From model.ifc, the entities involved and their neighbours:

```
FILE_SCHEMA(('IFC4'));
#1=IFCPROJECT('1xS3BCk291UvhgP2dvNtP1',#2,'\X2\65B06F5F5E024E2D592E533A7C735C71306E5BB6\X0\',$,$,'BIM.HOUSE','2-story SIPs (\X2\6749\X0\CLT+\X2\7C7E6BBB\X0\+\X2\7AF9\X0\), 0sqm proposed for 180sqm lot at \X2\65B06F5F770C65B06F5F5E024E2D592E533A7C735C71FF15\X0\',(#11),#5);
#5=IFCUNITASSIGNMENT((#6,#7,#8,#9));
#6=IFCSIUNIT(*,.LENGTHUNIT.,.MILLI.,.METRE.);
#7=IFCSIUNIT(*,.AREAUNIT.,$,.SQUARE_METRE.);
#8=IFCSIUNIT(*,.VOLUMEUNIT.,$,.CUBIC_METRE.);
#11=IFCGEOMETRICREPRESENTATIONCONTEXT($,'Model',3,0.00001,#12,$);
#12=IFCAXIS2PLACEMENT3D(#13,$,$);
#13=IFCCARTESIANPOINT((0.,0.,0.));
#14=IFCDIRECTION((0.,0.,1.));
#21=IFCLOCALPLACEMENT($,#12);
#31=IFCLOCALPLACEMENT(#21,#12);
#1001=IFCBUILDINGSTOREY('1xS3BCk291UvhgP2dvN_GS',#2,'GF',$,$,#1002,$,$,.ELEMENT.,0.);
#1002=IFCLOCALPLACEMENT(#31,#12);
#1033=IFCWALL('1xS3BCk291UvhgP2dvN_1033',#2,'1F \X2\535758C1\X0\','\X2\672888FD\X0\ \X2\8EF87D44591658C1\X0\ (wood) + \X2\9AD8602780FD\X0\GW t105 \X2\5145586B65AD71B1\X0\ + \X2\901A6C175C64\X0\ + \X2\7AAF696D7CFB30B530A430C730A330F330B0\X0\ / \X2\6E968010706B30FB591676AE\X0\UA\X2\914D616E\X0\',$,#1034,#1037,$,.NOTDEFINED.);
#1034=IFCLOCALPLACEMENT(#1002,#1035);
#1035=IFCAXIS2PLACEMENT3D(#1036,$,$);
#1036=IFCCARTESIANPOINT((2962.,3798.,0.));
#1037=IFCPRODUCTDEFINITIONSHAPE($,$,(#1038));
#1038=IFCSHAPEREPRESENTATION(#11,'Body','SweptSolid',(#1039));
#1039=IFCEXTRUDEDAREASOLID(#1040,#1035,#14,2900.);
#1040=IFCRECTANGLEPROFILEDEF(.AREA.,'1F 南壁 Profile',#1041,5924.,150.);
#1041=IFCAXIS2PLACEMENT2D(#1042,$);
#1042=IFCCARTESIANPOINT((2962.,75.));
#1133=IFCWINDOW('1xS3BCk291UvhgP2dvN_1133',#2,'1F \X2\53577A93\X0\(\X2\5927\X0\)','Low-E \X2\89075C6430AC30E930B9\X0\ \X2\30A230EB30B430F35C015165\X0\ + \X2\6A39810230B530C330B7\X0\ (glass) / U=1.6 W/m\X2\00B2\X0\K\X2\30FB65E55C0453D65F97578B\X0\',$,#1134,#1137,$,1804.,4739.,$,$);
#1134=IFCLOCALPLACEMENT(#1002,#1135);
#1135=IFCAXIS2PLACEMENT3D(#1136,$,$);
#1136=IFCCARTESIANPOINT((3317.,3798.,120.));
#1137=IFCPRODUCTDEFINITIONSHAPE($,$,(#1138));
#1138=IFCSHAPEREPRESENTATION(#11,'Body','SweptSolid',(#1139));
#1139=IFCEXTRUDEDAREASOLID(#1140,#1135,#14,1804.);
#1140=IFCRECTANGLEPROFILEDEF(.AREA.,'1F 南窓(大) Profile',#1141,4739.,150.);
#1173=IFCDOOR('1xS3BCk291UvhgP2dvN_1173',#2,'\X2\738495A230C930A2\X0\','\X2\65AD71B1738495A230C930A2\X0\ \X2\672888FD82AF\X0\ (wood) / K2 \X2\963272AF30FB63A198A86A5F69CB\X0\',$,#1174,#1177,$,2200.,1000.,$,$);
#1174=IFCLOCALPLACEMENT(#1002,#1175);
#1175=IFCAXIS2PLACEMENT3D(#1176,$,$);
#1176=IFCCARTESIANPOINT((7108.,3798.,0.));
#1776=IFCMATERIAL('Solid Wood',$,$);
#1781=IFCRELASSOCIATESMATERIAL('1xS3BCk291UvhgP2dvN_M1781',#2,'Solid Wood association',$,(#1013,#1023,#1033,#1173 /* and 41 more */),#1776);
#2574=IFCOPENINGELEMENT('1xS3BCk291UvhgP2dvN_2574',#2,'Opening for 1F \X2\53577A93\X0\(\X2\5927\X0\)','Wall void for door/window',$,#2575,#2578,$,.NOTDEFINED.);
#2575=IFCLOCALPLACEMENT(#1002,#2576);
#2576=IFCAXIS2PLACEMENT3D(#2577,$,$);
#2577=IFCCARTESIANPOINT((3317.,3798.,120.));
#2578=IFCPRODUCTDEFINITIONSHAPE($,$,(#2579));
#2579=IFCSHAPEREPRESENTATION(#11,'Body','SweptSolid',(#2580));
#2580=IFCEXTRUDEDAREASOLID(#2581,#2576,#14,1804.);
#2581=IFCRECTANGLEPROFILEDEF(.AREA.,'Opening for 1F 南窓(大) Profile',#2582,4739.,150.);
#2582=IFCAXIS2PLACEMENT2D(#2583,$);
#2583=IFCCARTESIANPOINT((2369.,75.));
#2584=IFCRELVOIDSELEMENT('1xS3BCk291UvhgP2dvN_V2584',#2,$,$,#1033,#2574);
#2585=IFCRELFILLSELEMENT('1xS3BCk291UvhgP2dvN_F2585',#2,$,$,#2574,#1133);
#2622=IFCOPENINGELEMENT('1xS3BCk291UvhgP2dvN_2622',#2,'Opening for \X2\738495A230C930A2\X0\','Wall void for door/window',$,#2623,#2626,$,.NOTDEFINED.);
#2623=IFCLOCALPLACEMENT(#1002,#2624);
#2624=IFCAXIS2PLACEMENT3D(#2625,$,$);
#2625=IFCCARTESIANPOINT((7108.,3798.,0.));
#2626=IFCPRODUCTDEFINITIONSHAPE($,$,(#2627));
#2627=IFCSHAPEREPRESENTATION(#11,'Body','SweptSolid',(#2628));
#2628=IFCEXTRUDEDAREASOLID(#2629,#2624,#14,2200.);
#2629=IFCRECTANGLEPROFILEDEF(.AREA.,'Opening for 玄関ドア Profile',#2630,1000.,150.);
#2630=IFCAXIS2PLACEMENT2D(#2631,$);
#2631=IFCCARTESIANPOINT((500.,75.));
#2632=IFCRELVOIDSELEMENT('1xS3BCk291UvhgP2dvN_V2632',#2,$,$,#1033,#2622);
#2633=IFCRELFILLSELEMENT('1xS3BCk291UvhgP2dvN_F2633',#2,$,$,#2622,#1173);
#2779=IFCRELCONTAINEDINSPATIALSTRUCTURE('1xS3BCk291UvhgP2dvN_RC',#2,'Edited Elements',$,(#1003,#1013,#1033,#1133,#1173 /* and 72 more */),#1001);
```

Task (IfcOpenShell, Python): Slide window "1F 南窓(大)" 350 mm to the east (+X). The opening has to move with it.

```python
import ifcopenshell
import ifcopenshell.api.geometry
import ifcopenshell.util.placement

model = ifcopenshell.open("model.ifc")

window = model.by_guid("1xS3BCk291UvhgP2dvN_1133")
opening = window.FillsVoids[0].RelatingOpeningElement
wall = opening.VoidsElements[0].RelatingBuildingElement

wall_matrix = ifcopenshell.util.placement.get_local_placement(wall.ObjectPlacement)
shift = wall_matrix[:3, 0] * 350.0
before = ifcopenshell.util.placement.get_local_placement(window.ObjectPlacement)[:3, 3].copy()

# The window is not placed relative to its opening, so move both.
for product in (opening, window):
    matrix = ifcopenshell.util.placement.get_local_placement(product.ObjectPlacement)
    matrix[:3, 3] += shift
    ifcopenshell.api.geometry.edit_object_placement(model, product=product, matrix=matrix, is_si=False)

after = ifcopenshell.util.placement.get_local_placement(window.ObjectPlacement)[:3, 3]
print("window moved by", (after - before).round(3) + 0.0)

model.write("model-out.ifc")
```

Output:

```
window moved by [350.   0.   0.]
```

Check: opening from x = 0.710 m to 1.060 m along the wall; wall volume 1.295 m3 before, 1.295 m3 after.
